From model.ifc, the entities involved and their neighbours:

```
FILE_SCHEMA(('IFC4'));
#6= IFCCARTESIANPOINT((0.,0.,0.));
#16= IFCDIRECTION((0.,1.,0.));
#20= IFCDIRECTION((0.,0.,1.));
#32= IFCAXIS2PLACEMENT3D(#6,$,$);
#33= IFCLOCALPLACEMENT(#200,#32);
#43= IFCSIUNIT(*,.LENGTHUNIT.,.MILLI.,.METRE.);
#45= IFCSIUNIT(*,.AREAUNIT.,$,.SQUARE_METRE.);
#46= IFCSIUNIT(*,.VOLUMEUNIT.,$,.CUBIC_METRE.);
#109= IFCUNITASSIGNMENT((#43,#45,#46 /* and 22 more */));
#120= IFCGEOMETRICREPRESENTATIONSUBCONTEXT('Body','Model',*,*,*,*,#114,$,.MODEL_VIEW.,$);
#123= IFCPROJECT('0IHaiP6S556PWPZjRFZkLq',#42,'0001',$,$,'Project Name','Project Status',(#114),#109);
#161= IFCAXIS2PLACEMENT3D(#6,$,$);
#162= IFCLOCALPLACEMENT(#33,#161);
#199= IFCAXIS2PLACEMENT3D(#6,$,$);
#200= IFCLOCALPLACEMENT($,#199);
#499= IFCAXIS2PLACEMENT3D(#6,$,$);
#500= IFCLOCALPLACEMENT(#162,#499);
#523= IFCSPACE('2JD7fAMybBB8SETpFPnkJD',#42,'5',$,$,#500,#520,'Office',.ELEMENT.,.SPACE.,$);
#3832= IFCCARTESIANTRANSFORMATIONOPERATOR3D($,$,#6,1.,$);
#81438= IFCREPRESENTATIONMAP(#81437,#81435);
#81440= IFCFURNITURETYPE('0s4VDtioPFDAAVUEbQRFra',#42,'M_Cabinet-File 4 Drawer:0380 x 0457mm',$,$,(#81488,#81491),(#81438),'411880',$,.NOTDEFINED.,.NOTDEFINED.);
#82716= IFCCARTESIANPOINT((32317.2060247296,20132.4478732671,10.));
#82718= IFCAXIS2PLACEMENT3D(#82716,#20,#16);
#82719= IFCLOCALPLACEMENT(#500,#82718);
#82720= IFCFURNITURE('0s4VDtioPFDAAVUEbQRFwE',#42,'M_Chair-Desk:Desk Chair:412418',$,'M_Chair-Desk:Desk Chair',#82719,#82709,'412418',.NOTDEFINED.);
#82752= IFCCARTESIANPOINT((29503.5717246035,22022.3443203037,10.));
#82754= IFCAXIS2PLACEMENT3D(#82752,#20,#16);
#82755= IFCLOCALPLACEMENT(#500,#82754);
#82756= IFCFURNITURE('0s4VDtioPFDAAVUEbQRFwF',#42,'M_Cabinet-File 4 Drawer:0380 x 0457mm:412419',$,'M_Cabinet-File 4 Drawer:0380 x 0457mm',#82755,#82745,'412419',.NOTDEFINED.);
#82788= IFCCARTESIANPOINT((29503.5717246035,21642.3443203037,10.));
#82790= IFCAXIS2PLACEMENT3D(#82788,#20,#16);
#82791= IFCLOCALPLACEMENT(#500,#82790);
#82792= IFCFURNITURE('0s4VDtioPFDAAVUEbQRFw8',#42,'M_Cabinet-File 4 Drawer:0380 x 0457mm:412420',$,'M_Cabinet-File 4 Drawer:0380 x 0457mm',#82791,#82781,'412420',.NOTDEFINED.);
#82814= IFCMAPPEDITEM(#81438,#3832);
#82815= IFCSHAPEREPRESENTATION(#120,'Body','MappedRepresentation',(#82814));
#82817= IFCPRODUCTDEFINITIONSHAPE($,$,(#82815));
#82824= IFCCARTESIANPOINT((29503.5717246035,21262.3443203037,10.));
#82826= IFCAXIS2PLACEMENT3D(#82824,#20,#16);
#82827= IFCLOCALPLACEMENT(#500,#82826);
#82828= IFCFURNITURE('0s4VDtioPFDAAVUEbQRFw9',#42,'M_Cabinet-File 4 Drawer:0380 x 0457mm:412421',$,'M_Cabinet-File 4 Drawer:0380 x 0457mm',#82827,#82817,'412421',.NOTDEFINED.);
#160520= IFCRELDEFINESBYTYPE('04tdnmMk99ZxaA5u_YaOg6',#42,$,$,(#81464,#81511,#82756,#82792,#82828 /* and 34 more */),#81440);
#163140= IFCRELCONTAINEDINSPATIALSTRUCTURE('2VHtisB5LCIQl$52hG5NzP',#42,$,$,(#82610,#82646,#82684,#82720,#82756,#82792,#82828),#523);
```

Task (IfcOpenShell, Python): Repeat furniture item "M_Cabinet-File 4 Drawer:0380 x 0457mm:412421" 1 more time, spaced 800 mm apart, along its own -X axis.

```python
import ifcopenshell
import ifcopenshell.api.geometry
import ifcopenshell.api.root
import ifcopenshell.util.element
import ifcopenshell.util.placement

model = ifcopenshell.open("model.ifc")


def reuse_history(source, copy):
    """copy_class also copies each property set's owner history, people and application; keep the originals."""
    for rel in copy.IsDefinedBy:
        if rel.is_a("IfcRelDefinesByProperties") and (history := rel.RelatingPropertyDefinition.OwnerHistory):
            rel.RelatingPropertyDefinition.OwnerHistory = source.OwnerHistory
            ifcopenshell.util.element.remove_deep2(model, history)


source = model.by_guid("0s4VDtioPFDAAVUEbQRFw9")
base = ifcopenshell.util.placement.get_local_placement(source.ObjectPlacement)
step = -base[:3, 0] * 800.0

for i in range(1, 2):
    copy = ifcopenshell.api.root.copy_class(model, product=source)
    copy.Representation = ifcopenshell.util.element.copy_deep(
        model, source.Representation, exclude=["IfcGeometricRepresentationContext", "IfcRepresentationMap"]
    )
    copy.Name = "M_Cabinet-File 4 Drawer:0380 x 0457mm"
    copy.Tag = None
    reuse_history(source, copy)
    matrix = base.copy()
    matrix[:3, 3] += i * step
    print("added at", matrix[:3, 3].round(3) + 0.0)
    ifcopenshell.api.geometry.edit_object_placement(model, product=copy, matrix=matrix, is_si=False)

model.write("model_rev.ifc")
```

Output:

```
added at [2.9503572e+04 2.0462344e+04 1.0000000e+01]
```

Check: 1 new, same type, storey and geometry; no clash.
